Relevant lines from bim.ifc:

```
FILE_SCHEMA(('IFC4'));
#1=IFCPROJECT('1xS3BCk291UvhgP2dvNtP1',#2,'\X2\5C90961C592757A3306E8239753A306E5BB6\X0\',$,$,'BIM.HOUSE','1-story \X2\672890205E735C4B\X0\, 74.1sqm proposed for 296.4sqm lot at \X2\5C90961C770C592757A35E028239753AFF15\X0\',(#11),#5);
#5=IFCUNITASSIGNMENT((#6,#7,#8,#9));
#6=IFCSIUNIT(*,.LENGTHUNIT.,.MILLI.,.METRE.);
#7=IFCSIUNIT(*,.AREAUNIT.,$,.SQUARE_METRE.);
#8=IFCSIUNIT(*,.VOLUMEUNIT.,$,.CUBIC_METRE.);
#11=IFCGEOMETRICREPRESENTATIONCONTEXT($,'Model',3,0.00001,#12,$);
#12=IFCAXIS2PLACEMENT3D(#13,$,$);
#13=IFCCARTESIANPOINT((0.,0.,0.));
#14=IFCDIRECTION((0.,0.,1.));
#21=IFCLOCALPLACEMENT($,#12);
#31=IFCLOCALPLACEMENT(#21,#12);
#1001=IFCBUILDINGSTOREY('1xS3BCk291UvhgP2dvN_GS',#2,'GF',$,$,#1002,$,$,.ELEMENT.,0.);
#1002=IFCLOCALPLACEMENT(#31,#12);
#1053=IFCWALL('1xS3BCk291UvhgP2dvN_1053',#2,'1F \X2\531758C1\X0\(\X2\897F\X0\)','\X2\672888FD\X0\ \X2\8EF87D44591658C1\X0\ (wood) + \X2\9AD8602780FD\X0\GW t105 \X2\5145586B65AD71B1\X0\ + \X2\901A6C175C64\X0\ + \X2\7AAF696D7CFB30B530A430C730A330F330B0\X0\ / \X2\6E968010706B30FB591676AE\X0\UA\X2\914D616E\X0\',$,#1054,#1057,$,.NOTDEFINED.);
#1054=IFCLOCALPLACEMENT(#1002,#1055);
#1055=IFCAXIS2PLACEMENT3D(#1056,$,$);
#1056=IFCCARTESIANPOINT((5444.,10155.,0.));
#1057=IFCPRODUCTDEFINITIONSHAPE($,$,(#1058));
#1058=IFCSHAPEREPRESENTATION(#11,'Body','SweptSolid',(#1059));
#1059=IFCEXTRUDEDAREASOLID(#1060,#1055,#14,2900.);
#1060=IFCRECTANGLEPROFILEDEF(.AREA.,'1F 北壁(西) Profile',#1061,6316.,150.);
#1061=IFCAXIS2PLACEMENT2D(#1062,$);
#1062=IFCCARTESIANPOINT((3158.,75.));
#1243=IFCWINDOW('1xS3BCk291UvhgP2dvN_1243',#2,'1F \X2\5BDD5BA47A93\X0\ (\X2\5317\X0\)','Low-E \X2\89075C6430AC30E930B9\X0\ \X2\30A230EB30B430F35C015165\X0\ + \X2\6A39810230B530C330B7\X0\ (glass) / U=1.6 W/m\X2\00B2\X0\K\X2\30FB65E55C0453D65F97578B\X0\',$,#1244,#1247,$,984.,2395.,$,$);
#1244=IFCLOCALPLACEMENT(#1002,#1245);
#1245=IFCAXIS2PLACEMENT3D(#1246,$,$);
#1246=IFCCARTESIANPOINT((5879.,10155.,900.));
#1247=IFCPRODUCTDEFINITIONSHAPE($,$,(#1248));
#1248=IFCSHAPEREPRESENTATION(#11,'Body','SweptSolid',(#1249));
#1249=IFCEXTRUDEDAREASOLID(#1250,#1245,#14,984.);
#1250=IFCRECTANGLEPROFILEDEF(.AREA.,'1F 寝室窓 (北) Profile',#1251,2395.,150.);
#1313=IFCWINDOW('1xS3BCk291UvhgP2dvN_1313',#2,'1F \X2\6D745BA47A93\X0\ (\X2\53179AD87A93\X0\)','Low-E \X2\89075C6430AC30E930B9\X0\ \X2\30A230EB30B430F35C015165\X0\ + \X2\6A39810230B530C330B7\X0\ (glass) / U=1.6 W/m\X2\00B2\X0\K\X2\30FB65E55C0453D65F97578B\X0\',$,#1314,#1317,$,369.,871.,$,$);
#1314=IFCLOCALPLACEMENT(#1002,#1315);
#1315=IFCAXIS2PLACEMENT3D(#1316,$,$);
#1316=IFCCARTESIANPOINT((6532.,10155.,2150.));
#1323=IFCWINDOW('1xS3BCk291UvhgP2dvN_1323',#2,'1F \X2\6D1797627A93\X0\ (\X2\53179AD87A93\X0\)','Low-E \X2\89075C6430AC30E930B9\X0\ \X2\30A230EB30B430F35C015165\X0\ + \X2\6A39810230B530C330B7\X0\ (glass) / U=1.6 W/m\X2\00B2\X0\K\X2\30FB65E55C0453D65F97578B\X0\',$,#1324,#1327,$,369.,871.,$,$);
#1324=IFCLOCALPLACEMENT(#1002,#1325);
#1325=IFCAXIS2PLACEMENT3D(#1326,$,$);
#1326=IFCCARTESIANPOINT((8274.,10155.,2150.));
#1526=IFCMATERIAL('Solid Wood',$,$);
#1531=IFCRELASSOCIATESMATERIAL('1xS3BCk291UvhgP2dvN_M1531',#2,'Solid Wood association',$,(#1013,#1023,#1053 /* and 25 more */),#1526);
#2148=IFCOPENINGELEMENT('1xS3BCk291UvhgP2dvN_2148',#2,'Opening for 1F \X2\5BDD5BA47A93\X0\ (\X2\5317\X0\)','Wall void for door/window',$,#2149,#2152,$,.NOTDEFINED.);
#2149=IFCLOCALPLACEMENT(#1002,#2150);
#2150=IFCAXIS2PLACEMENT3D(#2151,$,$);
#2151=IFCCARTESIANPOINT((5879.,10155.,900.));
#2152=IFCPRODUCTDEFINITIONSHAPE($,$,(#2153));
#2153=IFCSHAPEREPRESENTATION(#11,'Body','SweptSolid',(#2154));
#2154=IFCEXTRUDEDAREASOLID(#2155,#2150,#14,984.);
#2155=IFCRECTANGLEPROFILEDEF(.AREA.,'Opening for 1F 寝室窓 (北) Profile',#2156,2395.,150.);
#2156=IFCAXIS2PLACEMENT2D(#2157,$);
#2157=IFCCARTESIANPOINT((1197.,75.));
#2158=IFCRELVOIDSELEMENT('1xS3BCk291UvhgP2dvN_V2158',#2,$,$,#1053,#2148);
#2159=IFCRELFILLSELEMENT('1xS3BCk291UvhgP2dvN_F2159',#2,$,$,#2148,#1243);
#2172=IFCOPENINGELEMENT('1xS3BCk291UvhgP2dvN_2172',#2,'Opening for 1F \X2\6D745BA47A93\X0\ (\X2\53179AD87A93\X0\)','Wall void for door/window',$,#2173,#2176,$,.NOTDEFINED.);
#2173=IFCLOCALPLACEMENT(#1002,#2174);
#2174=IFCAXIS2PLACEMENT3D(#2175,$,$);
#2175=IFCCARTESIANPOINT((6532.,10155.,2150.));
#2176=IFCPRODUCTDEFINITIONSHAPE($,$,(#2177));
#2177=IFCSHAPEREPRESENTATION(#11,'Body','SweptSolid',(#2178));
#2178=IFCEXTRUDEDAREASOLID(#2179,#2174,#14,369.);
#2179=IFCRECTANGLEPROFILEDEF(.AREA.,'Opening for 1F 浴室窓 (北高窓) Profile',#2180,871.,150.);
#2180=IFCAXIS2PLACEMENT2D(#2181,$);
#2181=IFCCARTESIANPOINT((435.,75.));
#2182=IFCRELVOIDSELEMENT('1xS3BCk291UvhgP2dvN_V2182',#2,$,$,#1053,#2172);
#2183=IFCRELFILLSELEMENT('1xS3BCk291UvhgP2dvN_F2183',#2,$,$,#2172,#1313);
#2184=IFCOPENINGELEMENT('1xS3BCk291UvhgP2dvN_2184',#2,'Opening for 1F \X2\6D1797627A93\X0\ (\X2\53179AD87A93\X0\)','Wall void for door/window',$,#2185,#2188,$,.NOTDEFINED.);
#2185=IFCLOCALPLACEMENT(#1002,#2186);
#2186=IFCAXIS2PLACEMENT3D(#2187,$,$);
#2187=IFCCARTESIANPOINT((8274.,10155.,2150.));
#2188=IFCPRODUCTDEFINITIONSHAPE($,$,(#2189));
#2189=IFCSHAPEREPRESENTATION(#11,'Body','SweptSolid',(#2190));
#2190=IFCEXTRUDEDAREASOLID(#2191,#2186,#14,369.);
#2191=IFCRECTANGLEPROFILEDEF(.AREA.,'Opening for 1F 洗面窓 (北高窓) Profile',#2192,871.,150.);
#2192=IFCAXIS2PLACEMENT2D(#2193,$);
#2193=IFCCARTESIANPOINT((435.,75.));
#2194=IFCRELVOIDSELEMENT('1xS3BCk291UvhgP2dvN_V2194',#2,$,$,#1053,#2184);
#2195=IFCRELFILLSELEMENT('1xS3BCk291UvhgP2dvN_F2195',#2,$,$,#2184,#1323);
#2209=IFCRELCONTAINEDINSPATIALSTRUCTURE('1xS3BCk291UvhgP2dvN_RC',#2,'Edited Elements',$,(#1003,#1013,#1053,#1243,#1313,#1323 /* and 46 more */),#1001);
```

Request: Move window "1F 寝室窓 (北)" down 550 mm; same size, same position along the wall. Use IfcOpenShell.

```python
import numpy as np
import ifcopenshell
import ifcopenshell.api.geometry
import ifcopenshell.util.placement
import ifcopenshell.util.unit

model = ifcopenshell.open("bim.ifc")
unit_scale = ifcopenshell.util.unit.calculate_unit_scale(model)

window = model.by_id(1243)
opening = window.FillsVoids[0].RelatingOpeningElement
dz = -550.0

shift = np.array([0.0, 0.0, dz])
# The window is not placed relative to its opening, so move both.
for product in (opening, window):
    matrix = ifcopenshell.util.placement.get_local_placement(product.ObjectPlacement)
    matrix[:3, 3] += shift
    ifcopenshell.api.geometry.edit_object_placement(model, product=product, matrix=matrix, is_si=False)

print(f"moved by {dz * unit_scale:+.3f} m")

model.write("bim_updated.ifc")
```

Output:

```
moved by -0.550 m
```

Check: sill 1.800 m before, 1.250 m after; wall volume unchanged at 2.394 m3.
